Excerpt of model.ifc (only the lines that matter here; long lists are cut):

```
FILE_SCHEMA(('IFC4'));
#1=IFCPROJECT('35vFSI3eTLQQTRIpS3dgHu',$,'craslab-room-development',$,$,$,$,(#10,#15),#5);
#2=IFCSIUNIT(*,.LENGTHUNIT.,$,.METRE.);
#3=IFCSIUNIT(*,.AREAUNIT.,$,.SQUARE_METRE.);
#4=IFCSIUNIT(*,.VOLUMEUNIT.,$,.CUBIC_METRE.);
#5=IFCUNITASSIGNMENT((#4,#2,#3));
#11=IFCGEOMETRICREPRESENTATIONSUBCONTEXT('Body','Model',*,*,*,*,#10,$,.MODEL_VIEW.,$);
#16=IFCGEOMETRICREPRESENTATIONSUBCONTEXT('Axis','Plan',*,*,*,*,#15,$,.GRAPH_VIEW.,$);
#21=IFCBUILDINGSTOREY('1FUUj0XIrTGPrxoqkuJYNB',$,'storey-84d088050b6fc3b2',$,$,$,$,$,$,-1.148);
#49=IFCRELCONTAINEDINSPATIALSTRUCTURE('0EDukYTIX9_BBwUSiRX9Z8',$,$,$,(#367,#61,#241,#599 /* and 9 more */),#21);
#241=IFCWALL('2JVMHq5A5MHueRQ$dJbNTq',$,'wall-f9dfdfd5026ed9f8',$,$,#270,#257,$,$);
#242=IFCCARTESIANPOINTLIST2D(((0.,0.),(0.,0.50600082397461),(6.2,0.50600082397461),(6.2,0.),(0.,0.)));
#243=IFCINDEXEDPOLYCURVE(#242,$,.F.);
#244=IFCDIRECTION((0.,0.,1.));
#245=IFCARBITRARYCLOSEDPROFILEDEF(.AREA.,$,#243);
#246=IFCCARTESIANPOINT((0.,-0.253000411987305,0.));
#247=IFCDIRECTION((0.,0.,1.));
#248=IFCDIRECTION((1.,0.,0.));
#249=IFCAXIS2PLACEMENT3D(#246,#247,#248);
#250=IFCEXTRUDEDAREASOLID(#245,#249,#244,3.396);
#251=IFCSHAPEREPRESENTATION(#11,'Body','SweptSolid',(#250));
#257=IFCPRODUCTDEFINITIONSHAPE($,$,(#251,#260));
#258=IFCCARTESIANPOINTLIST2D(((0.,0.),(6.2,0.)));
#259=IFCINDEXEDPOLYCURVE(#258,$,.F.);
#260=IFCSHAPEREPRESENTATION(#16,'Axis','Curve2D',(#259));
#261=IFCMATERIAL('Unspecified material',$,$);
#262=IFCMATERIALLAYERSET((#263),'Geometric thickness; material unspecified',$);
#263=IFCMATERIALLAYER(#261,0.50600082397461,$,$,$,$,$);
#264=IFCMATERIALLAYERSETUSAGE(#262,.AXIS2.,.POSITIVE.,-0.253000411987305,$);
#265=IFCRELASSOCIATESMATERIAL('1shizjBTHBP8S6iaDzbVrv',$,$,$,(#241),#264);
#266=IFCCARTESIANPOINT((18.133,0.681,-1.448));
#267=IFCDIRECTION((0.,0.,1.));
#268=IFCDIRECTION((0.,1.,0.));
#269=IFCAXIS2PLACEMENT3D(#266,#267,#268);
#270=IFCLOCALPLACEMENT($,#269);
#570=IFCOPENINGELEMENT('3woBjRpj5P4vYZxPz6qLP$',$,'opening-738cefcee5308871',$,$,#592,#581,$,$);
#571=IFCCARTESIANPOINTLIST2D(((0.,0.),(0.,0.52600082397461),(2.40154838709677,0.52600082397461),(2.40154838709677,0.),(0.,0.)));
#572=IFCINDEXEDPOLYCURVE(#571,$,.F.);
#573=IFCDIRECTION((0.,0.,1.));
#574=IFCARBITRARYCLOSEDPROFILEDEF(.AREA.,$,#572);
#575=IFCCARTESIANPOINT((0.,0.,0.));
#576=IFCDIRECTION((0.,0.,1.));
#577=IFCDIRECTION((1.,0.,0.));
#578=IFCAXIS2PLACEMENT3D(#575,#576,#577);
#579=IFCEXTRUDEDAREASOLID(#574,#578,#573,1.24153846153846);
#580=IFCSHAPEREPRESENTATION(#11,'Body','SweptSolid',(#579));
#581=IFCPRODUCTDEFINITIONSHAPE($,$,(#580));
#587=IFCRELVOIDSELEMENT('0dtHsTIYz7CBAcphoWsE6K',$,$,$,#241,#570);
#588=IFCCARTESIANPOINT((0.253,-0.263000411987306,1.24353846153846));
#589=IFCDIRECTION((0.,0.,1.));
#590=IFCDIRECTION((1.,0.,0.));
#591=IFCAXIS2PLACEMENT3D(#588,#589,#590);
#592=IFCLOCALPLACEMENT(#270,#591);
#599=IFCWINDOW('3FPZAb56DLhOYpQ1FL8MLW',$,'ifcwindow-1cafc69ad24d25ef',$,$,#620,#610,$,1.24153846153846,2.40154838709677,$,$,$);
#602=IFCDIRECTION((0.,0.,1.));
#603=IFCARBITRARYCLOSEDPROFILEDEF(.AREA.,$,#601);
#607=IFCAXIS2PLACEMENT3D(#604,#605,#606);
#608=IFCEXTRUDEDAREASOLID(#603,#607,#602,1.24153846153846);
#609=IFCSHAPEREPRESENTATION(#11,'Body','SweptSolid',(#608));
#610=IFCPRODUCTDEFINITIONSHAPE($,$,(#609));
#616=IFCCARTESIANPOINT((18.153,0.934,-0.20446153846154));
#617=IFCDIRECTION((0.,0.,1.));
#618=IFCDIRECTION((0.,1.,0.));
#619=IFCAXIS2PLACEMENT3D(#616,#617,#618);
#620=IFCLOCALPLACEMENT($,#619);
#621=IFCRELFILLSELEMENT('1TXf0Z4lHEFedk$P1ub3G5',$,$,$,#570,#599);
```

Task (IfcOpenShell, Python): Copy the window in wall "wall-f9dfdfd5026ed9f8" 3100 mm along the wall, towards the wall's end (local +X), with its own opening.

```python
import ifcopenshell
import ifcopenshell.api.feature
import ifcopenshell.api.geometry
import ifcopenshell.api.root
import ifcopenshell.geom
import ifcopenshell.util.element
import ifcopenshell.util.placement
import ifcopenshell.util.shape
import ifcopenshell.util.unit

model = ifcopenshell.open("model.ifc")
unit_scale = ifcopenshell.util.unit.calculate_unit_scale(model)
settings = ifcopenshell.geom.settings()


def volume(element):
    """Net volume in cubic metres, openings subtracted."""
    shape = ifcopenshell.geom.create_shape(settings, element)
    return ifcopenshell.util.shape.get_volume(shape.geometry)


window = model.by_guid("3FPZAb56DLhOYpQ1FL8MLW")
opening = window.FillsVoids[0].RelatingOpeningElement
wall = opening.VoidsElements[0].RelatingBuildingElement
before = volume(wall)
shift = ifcopenshell.util.placement.get_local_placement(wall.ObjectPlacement)[:3, 0] * 3.1 / unit_scale

# copy_class copies the void relationship, type, container and properties, but no geometry.
new_opening = ifcopenshell.api.root.copy_class(model, product=opening)
new_opening.Representation = ifcopenshell.util.element.copy_deep(
    model, opening.Representation, exclude=["IfcGeometricRepresentationContext", "IfcRepresentationMap"]
)
new_window = ifcopenshell.api.root.copy_class(model, product=window)
new_window.Representation = ifcopenshell.util.element.copy_deep(
    model, window.Representation, exclude=["IfcGeometricRepresentationContext", "IfcRepresentationMap"]
)
ifcopenshell.api.feature.add_filling(model, opening=new_opening, element=new_window)

for old, new in ((opening, new_opening), (window, new_window)):
    matrix = ifcopenshell.util.placement.get_local_placement(old.ObjectPlacement)
    matrix[:3, 3] += shift
    ifcopenshell.api.geometry.edit_object_placement(model, product=new, matrix=matrix, is_si=False)

after = volume(wall)

print(f"wall volume {before:.3f} -> {after:.3f} m3")

model.write("model_v2.ifc")
```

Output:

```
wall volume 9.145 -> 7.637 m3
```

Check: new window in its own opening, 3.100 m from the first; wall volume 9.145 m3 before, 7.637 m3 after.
